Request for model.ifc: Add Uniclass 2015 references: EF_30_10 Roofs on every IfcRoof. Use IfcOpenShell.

First a look at what the model holds.

```python
import ifcopenshell

model = ifcopenshell.open("model.ifc")
print(model.schema)
print("classifications:", [c.Name for c in model.by_type("IfcClassification")])
for ifc_class in ("IfcDoor", "IfcRoof", "IfcStair", "IfcWall", "IfcWindow"):
    print(ifc_class, len(model.by_type(ifc_class)))
```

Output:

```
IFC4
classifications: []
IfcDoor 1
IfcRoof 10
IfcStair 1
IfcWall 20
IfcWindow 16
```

```python
import ifcopenshell
import ifcopenshell.api.classification

model = ifcopenshell.open("model.ifc")

system = ifcopenshell.api.classification.add_classification(model, classification="Uniclass 2015")

codes = {
    "IfcRoof": ("EF_30_10", "Roofs"),
}
for ifc_class, (code, name) in codes.items():
    products = model.by_type(ifc_class)
    ifcopenshell.api.classification.add_reference(
        model, products=products, classification=system, identification=code, name=name
    )
    print(code, len(products))

model.write("model_rev.ifc")
```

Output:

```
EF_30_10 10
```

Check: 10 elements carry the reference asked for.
